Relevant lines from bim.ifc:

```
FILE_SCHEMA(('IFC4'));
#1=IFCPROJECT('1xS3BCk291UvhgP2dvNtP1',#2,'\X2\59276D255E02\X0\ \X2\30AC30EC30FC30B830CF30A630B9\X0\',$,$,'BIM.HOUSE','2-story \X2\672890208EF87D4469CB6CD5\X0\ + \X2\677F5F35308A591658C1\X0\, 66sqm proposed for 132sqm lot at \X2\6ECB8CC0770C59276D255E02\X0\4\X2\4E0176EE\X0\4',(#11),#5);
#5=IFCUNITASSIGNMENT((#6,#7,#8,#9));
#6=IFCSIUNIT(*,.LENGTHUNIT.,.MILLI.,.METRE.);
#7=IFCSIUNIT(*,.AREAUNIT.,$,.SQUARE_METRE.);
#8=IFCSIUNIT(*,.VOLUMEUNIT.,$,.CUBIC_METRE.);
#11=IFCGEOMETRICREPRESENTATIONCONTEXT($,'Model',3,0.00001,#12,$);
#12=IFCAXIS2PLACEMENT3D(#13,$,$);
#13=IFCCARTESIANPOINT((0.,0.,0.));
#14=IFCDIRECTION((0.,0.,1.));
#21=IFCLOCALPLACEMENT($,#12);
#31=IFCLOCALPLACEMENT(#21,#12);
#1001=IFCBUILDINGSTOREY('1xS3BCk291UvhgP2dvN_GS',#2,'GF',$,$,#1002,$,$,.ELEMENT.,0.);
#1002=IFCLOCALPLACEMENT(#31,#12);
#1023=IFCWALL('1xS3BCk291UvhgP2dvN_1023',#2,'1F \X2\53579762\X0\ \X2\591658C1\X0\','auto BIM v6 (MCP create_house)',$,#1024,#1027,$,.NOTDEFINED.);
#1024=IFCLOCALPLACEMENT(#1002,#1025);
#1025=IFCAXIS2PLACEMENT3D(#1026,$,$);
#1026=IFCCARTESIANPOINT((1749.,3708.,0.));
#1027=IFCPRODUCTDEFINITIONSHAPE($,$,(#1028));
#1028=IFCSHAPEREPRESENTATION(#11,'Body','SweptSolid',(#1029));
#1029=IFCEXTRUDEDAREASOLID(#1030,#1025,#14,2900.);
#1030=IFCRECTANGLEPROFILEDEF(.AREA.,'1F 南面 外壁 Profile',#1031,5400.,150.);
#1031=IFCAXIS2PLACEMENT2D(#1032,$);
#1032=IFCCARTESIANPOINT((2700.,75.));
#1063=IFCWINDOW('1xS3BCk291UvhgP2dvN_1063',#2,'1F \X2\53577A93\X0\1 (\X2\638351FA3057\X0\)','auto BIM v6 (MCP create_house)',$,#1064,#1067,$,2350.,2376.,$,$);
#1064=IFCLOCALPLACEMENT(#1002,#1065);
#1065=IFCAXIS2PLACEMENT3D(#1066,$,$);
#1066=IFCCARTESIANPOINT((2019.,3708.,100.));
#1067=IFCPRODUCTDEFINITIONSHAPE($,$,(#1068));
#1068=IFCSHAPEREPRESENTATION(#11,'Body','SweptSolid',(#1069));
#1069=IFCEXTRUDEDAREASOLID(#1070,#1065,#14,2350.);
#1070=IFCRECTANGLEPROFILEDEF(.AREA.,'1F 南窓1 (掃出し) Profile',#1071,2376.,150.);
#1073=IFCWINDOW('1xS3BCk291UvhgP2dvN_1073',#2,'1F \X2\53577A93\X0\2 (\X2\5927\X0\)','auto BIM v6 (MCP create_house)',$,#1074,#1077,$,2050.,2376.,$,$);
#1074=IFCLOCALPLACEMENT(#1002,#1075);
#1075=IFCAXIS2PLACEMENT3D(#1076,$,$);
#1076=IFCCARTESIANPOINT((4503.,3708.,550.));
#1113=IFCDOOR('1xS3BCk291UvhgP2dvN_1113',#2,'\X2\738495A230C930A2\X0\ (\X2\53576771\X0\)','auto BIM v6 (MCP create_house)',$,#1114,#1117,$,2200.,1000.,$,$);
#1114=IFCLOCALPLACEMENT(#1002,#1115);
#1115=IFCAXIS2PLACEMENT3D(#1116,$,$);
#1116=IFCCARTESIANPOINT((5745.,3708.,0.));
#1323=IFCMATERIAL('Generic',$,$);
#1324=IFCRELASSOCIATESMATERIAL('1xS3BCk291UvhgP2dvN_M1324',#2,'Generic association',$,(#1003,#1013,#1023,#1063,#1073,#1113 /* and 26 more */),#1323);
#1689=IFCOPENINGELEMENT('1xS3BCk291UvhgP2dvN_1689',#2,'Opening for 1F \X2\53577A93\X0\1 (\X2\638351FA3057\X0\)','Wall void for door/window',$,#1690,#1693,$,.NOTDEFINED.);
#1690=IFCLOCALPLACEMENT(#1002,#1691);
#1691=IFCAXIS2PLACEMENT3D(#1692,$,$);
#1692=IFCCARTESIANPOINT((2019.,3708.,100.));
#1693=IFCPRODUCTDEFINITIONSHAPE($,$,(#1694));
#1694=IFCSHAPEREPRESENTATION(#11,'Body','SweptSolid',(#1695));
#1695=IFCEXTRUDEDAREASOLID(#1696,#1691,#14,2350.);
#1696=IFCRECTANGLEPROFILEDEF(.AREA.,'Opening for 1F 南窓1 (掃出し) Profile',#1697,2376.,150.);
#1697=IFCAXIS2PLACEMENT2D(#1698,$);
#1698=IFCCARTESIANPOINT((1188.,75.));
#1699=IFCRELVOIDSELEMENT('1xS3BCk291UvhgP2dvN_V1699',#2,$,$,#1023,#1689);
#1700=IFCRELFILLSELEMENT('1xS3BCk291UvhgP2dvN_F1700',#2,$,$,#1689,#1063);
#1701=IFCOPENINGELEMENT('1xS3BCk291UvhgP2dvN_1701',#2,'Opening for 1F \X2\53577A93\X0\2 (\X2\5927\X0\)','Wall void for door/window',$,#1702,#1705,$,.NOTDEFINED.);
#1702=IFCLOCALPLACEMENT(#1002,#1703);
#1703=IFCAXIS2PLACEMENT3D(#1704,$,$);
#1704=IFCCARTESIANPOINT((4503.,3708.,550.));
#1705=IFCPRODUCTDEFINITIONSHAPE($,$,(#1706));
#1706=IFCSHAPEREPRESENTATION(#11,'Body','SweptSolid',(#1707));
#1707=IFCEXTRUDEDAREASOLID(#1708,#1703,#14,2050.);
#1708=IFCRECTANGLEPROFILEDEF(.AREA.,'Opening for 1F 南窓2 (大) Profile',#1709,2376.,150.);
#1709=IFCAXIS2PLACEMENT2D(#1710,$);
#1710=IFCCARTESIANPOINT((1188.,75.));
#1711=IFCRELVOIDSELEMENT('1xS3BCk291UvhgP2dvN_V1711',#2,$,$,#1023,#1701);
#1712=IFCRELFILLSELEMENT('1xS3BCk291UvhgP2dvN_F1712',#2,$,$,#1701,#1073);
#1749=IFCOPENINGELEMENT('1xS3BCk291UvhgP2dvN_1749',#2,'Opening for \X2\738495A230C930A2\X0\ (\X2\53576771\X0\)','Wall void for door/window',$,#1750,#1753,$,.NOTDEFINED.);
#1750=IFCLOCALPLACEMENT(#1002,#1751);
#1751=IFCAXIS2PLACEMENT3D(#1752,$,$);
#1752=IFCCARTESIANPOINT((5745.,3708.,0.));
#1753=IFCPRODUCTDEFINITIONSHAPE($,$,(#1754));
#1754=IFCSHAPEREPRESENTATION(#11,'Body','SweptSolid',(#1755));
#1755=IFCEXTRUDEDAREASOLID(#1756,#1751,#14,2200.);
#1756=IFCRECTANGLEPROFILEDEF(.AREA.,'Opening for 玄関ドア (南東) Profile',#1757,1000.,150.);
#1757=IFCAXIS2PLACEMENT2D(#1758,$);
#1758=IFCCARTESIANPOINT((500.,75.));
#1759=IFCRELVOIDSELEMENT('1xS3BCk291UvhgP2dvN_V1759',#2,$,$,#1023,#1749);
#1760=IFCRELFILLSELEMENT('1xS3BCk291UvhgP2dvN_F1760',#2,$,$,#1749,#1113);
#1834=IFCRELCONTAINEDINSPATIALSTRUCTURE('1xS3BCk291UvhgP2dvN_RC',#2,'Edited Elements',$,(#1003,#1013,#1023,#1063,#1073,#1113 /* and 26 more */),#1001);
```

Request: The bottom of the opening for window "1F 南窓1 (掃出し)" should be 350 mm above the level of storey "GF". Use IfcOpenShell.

```python
import numpy as np
import ifcopenshell
import ifcopenshell.api.geometry
import ifcopenshell.geom
import ifcopenshell.util.element
import ifcopenshell.util.placement
import ifcopenshell.util.shape
import ifcopenshell.util.unit

model = ifcopenshell.open("bim.ifc")
unit_scale = ifcopenshell.util.unit.calculate_unit_scale(model)

window = model.by_guid("1xS3BCk291UvhgP2dvN_1063")
opening = window.FillsVoids[0].RelatingOpeningElement
storey = ifcopenshell.util.element.get_container(window, ifc_class="IfcBuildingStorey")
level = ifcopenshell.util.placement.get_local_placement(storey.ObjectPlacement)[2, 3]

# The opening's origin need not be at the sill, so measure its lowest point.
shape = ifcopenshell.geom.create_shape(ifcopenshell.geom.settings(), opening)
bottom = ifcopenshell.util.shape.get_shape_bottom_elevation(shape, shape.geometry) / unit_scale
dz = level + 0.35 / unit_scale - bottom

shift = np.array([0.0, 0.0, dz])
# The window is not placed relative to its opening, so move both.
for product in (opening, window):
    matrix = ifcopenshell.util.placement.get_local_placement(product.ObjectPlacement)
    matrix[:3, 3] += shift
    ifcopenshell.api.geometry.edit_object_placement(model, product=product, matrix=matrix, is_si=False)

print(f"moved by {dz * unit_scale:+.3f} m")

model.write("bim_rev.ifc")
```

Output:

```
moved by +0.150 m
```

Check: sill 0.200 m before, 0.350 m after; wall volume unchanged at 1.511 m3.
